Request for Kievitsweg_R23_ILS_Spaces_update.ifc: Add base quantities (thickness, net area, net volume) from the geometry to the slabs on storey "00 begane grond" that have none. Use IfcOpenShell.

First a look at what the model holds.

```python
import ifcopenshell
import ifcopenshell.util.element
import ifcopenshell.util.unit

model = ifcopenshell.open("Kievitsweg_R23_ILS_Spaces_update.ifc")
print(model.schema)
for unit_type in ("LENGTHUNIT", "AREAUNIT", "VOLUMEUNIT"):
    print(unit_type, ifcopenshell.util.unit.calculate_unit_scale(model, unit_type))
storey = next(s for s in model.by_type("IfcBuildingStorey") if s.Name == "00 begane grond")
slabs = [e for e in ifcopenshell.util.element.get_decomposition(storey) if e.is_a("IfcSlab")]
for e in sorted(slabs, key=lambda e: e.id()):
    print(e.id(), e.is_a(), e.Name, list(ifcopenshell.util.element.get_psets(e, qtos_only=True)), sep=" | ")
```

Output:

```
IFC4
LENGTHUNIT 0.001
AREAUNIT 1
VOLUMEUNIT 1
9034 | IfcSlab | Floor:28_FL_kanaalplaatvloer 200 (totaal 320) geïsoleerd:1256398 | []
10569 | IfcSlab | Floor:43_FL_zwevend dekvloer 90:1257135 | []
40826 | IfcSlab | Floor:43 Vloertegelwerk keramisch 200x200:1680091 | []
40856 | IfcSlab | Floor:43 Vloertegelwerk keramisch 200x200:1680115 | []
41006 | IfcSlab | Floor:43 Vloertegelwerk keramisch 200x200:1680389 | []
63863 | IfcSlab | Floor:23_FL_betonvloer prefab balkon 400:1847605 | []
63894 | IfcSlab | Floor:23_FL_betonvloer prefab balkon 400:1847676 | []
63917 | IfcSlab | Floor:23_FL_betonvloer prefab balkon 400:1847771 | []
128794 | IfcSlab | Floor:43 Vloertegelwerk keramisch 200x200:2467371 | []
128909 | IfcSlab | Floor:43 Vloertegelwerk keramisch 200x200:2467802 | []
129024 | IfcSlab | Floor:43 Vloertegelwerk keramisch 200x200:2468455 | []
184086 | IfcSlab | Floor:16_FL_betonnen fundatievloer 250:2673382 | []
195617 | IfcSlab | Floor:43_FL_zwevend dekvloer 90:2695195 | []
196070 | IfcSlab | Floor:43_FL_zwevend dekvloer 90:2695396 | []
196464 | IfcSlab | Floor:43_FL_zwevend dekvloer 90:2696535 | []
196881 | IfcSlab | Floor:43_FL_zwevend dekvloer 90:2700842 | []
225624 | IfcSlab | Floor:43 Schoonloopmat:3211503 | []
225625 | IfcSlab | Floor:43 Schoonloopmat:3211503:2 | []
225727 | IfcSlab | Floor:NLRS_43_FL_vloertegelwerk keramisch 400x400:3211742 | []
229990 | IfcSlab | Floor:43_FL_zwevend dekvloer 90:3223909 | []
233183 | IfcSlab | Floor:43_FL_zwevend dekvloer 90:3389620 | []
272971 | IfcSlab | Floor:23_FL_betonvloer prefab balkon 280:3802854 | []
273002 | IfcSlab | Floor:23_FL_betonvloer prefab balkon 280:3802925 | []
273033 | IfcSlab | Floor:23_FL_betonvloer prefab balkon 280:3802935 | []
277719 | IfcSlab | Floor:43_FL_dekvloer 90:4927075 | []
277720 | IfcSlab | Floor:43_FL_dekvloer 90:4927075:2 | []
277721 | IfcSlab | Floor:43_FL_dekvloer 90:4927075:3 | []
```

```python
import ifcopenshell
import ifcopenshell.api.pset
import ifcopenshell.geom
import ifcopenshell.util.element
import ifcopenshell.util.shape
import ifcopenshell.util.unit

model = ifcopenshell.open("Kievitsweg_R23_ILS_Spaces_update.ifc")
unit_scale = ifcopenshell.util.unit.calculate_unit_scale(model)
area_scale = ifcopenshell.util.unit.calculate_unit_scale(model, "AREAUNIT")
volume_scale = ifcopenshell.util.unit.calculate_unit_scale(model, "VOLUMEUNIT")
settings = ifcopenshell.geom.settings()

storey = next(s for s in model.by_type("IfcBuildingStorey") if s.Name == "00 begane grond")
slabs = [e for e in ifcopenshell.util.element.get_decomposition(storey) if e.is_a("IfcSlab")]

for e in sorted(slabs, key=lambda e: e.id()):
    if ifcopenshell.util.element.get_psets(e, qtos_only=True, should_inherit=False):
        continue
    # Geometry comes back in metres, in the element's own axes.
    shape = ifcopenshell.geom.create_shape(settings, e)
    values = {
        "Width": ifcopenshell.util.shape.get_z(shape.geometry) / unit_scale,
        "NetArea": ifcopenshell.util.shape.get_footprint_area(shape.geometry) / area_scale,
        "NetVolume": ifcopenshell.util.shape.get_volume(shape.geometry) / volume_scale,
    }
    qto = ifcopenshell.api.pset.add_qto(model, product=e, name="Qto_SlabBaseQuantities")
    ifcopenshell.api.pset.edit_qto(model, qto=qto, properties=values)
    print(e.id(), {k: round(v, 3) for k, v in values.items()})

model.write("Kievitsweg_R23_ILS_Spaces_update_rev.ifc")
```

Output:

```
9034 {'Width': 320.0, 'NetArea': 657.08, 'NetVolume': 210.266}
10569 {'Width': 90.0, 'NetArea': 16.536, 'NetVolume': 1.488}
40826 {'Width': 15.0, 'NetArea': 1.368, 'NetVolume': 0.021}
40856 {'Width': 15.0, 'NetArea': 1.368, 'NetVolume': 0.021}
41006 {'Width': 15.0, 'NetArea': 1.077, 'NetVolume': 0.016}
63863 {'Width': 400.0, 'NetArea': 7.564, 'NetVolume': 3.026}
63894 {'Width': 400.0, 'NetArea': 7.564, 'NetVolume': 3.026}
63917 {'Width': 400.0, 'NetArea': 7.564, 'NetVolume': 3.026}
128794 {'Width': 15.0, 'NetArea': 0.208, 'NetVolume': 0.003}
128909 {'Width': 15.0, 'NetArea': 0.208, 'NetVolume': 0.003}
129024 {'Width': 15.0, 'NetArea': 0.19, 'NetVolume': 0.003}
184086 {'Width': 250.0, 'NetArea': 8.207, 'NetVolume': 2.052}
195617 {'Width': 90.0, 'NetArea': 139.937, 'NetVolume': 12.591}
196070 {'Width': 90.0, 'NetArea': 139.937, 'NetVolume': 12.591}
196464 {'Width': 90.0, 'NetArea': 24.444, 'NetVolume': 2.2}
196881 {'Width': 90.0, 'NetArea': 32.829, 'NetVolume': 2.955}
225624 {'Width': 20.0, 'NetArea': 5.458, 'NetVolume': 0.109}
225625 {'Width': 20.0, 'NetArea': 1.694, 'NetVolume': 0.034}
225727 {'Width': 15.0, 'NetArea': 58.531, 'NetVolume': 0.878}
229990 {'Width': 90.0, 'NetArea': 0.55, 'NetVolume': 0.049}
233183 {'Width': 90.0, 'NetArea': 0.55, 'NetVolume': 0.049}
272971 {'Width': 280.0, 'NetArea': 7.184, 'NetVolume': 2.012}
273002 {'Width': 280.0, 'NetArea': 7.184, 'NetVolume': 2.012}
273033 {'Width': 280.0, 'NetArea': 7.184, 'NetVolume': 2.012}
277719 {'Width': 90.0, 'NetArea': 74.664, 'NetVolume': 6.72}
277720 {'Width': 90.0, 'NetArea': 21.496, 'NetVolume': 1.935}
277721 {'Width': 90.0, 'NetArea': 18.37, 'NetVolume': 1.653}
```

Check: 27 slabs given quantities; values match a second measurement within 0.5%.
